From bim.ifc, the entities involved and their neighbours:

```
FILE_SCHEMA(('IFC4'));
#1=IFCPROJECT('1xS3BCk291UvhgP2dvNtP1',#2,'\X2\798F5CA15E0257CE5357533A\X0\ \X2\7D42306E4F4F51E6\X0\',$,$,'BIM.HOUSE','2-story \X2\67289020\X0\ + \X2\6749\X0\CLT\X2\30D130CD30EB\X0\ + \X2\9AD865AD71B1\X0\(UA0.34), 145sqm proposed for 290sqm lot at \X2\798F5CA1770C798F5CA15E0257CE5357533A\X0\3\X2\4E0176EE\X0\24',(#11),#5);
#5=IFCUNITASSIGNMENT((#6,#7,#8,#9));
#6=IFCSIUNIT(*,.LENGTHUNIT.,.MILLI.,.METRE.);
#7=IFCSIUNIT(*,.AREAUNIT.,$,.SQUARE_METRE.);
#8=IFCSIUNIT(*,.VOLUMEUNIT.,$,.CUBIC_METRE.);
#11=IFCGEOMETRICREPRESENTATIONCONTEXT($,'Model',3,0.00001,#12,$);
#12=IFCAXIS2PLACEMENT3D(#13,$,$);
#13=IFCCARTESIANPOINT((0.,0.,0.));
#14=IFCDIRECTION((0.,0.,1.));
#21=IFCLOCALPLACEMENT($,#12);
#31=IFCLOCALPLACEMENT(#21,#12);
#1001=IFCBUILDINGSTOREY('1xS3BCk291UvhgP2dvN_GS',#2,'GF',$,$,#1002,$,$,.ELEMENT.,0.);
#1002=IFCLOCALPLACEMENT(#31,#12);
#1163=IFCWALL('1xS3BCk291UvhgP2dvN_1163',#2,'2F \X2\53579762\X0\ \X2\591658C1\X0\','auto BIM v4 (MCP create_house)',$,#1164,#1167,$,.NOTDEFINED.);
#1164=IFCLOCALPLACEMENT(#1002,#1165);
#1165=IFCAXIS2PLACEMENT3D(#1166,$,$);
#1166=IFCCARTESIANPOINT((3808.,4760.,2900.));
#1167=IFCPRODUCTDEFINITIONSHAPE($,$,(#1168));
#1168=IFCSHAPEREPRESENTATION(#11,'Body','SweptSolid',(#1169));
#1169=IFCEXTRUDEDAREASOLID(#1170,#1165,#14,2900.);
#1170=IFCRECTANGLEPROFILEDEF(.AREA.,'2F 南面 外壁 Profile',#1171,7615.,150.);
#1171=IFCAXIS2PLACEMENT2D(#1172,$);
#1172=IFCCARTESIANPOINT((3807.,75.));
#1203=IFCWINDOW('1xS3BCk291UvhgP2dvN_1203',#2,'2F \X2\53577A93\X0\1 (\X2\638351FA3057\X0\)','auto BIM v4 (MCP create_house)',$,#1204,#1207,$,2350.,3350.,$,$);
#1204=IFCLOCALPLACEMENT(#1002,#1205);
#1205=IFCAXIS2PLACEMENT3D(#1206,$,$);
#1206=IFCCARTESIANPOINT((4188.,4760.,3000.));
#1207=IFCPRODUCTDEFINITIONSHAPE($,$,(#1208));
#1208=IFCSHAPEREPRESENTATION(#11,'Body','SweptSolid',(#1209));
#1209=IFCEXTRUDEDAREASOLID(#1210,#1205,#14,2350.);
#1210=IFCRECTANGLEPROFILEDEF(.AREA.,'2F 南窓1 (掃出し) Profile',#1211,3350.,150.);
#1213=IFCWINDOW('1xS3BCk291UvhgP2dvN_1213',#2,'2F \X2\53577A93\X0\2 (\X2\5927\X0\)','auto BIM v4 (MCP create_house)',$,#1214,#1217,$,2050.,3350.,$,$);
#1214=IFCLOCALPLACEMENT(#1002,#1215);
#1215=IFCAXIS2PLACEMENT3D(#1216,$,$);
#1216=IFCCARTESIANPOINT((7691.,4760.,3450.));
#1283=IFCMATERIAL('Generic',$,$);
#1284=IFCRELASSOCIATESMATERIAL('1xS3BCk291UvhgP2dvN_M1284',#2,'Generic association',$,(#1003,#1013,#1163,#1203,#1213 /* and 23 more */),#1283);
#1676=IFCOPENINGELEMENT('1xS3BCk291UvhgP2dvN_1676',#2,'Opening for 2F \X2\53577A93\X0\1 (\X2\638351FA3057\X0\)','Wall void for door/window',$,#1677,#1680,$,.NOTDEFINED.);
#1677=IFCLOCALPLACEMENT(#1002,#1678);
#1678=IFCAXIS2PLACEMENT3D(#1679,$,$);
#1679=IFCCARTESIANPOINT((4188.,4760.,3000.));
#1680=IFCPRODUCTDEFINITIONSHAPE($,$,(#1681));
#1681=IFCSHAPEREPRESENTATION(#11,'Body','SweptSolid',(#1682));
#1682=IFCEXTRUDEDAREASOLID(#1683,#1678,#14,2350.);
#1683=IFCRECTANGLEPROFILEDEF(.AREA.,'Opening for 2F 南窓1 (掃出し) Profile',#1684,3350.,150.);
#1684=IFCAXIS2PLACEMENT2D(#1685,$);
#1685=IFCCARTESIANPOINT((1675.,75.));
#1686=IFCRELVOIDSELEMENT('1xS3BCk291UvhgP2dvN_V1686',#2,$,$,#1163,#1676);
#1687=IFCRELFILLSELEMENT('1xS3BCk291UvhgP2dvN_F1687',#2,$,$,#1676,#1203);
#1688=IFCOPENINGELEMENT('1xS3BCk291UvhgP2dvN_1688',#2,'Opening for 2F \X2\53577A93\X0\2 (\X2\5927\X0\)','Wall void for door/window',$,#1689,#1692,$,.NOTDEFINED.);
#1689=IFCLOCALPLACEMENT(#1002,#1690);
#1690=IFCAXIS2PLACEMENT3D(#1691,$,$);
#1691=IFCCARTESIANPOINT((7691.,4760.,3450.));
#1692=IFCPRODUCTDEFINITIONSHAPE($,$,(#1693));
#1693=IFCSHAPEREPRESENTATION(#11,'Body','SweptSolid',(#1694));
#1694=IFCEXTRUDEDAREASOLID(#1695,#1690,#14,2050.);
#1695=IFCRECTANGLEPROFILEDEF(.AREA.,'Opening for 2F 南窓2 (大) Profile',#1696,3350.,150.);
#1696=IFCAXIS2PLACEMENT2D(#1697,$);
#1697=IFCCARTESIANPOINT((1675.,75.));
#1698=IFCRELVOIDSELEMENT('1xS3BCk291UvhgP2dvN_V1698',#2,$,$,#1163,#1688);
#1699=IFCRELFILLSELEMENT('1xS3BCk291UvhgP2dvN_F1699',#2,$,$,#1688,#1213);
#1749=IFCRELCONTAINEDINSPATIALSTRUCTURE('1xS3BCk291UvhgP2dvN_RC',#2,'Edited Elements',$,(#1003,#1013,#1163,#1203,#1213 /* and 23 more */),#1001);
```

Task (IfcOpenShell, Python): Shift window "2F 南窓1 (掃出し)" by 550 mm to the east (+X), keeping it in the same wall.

```python
import ifcopenshell
import ifcopenshell.api.geometry
import ifcopenshell.util.placement
import ifcopenshell.util.unit

model = ifcopenshell.open("bim.ifc")
unit_scale = ifcopenshell.util.unit.calculate_unit_scale(model)

window = model.by_id(1203)
opening = window.FillsVoids[0].RelatingOpeningElement
wall = opening.VoidsElements[0].RelatingBuildingElement

wall_matrix = ifcopenshell.util.placement.get_local_placement(wall.ObjectPlacement)
shift = wall_matrix[:3, 0] * 0.55 / unit_scale
before = ifcopenshell.util.placement.get_local_placement(window.ObjectPlacement)[:3, 3].copy()

# The window is not placed relative to its opening, so move both.
for product in (opening, window):
    matrix = ifcopenshell.util.placement.get_local_placement(product.ObjectPlacement)
    matrix[:3, 3] += shift
    ifcopenshell.api.geometry.edit_object_placement(model, product=product, matrix=matrix, is_si=False)

after = ifcopenshell.util.placement.get_local_placement(window.ObjectPlacement)[:3, 3]
print("window moved by", (after - before).round(3) + 0.0)

model.write("bim_updated.ifc")
```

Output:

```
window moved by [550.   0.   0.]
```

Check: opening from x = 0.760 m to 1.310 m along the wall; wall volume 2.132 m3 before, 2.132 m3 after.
